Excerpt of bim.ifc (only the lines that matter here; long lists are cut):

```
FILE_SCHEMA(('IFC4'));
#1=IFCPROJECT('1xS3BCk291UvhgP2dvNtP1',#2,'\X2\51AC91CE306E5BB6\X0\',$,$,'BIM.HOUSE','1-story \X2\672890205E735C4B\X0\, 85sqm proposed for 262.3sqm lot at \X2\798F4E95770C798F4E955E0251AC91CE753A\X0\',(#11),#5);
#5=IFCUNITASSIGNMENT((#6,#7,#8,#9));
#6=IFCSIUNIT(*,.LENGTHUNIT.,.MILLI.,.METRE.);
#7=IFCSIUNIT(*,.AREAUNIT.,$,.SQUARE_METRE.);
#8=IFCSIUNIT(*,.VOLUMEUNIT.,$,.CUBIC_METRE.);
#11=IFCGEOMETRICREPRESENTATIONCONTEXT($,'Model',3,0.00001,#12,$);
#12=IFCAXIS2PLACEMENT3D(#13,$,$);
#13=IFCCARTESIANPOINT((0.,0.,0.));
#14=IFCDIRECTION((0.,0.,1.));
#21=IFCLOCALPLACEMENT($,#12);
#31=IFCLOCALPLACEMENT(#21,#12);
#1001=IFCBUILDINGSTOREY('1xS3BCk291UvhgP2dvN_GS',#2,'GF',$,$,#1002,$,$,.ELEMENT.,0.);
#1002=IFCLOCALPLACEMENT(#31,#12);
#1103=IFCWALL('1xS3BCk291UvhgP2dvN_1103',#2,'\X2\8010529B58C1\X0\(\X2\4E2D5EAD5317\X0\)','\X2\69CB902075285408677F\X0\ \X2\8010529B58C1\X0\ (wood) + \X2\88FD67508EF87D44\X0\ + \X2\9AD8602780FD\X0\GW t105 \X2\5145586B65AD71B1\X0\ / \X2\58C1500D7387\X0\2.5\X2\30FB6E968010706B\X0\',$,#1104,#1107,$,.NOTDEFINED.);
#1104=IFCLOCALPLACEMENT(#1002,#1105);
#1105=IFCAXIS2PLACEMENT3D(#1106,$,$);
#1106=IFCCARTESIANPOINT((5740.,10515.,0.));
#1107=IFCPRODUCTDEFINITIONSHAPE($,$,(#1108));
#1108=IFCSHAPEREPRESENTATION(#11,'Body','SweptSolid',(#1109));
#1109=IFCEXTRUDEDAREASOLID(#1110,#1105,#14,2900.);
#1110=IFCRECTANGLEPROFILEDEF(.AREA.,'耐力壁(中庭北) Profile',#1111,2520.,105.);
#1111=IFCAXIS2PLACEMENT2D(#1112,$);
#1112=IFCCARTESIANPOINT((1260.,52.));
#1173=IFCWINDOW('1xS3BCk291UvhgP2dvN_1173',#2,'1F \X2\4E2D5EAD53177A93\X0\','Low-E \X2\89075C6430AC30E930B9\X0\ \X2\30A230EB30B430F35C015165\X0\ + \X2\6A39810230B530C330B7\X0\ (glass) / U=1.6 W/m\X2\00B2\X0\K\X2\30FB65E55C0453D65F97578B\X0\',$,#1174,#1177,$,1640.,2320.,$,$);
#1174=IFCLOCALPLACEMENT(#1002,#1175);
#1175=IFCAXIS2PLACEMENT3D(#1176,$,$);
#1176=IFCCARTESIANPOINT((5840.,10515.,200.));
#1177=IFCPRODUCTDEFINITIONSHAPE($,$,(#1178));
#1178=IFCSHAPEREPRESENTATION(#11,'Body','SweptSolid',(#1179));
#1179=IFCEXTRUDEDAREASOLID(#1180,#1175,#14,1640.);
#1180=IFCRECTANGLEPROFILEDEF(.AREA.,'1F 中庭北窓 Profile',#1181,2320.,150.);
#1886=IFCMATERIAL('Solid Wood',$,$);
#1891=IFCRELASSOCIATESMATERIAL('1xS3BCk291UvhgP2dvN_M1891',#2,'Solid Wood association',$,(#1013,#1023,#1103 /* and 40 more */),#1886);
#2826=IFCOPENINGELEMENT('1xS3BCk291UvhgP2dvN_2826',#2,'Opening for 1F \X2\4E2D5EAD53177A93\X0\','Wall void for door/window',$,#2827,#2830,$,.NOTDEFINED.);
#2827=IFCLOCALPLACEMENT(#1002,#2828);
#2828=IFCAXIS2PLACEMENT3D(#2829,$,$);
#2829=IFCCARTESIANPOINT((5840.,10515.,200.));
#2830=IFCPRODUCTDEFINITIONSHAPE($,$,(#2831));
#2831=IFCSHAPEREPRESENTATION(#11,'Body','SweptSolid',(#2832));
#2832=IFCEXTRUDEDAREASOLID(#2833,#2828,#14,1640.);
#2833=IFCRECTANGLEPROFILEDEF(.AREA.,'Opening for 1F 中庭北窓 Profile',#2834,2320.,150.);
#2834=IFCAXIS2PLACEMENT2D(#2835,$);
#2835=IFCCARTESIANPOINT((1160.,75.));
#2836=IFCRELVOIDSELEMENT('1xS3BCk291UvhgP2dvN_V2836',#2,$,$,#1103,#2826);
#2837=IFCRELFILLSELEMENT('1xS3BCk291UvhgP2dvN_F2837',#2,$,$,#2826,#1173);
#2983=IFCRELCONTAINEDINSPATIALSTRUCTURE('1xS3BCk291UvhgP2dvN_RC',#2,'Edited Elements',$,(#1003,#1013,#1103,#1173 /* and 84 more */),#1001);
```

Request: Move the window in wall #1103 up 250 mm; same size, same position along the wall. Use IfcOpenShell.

```python
import numpy as np
import ifcopenshell
import ifcopenshell.api.geometry
import ifcopenshell.util.placement
import ifcopenshell.util.unit

model = ifcopenshell.open("bim.ifc")
unit_scale = ifcopenshell.util.unit.calculate_unit_scale(model)

window = model.by_guid("1xS3BCk291UvhgP2dvN_1173")
opening = window.FillsVoids[0].RelatingOpeningElement
dz = 250.0

shift = np.array([0.0, 0.0, dz])
# The window is not placed relative to its opening, so move both.
for product in (opening, window):
    matrix = ifcopenshell.util.placement.get_local_placement(product.ObjectPlacement)
    matrix[:3, 3] += shift
    ifcopenshell.api.geometry.edit_object_placement(model, product=product, matrix=matrix, is_si=False)

print(f"moved by {dz * unit_scale:+.3f} m")

model.write("bim-out.ifc")
```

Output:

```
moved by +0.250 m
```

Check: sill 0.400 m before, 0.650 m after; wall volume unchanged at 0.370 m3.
